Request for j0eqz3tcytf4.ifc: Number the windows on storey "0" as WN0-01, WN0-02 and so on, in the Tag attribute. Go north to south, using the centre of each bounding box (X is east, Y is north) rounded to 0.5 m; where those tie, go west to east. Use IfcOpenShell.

First a look at what the model holds.

```python
import ifcopenshell
import ifcopenshell.util.element
import ifcopenshell.util.placement

model = ifcopenshell.open("j0eqz3tcytf4.ifc")
print(model.schema)
storey = next(s for s in model.by_type("IfcBuildingStorey") if s.Name == "0")
windows = [e for e in ifcopenshell.util.element.get_decomposition(storey) if e.is_a("IfcWindow")]
for e in sorted(windows, key=lambda e: e.id()):
    origin = ifcopenshell.util.placement.get_local_placement(e.ObjectPlacement)[:3, 3]
    print(e.id(), e.Tag, e.Name, origin.round(2) + 0.0, sep=" | ")
```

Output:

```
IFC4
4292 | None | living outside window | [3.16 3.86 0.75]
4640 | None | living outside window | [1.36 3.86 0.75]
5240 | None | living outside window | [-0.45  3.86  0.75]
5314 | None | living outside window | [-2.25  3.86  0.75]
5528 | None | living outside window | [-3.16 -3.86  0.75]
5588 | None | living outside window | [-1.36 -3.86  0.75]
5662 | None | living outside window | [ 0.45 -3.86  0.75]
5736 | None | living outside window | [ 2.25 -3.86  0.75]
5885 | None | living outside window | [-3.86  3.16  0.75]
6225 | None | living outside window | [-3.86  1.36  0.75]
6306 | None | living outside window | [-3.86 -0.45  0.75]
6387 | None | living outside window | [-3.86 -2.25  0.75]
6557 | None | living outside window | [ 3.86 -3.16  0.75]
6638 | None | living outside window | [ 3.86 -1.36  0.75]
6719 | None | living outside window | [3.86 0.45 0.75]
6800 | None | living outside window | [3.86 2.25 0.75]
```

```python
import ifcopenshell
import ifcopenshell.geom
import ifcopenshell.util.element
import ifcopenshell.util.shape

model = ifcopenshell.open("j0eqz3tcytf4.ifc")
settings = ifcopenshell.geom.settings()
settings.set("use-world-coords", True)


def centre(element):
    shape = ifcopenshell.geom.create_shape(settings, element)
    return ifcopenshell.util.shape.get_bbox_centroid(shape.geometry)


storey = next(s for s in model.by_type("IfcBuildingStorey") if s.Name == "0")
windows = [e for e in ifcopenshell.util.element.get_decomposition(storey) if e.is_a("IfcWindow")]

# Insertion points can sit at a corner or the storey origin, so sort by the geometry (in metres).
centres = {e: centre(e) for e in windows}
windows.sort(key=lambda e: (-round(centres[e][1] / 0.5), centres[e][0]))

for i, e in enumerate(windows, start=1):
    number = f"WN0-{i:02d}"
    e.Tag = number
    print(e.id(), number)

model.write("j0eqz3tcytf4_updated.ifc")
```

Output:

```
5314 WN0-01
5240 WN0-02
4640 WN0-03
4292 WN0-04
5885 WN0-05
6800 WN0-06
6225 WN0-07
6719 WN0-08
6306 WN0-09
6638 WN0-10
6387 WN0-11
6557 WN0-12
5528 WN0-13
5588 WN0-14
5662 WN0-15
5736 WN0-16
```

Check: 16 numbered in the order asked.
